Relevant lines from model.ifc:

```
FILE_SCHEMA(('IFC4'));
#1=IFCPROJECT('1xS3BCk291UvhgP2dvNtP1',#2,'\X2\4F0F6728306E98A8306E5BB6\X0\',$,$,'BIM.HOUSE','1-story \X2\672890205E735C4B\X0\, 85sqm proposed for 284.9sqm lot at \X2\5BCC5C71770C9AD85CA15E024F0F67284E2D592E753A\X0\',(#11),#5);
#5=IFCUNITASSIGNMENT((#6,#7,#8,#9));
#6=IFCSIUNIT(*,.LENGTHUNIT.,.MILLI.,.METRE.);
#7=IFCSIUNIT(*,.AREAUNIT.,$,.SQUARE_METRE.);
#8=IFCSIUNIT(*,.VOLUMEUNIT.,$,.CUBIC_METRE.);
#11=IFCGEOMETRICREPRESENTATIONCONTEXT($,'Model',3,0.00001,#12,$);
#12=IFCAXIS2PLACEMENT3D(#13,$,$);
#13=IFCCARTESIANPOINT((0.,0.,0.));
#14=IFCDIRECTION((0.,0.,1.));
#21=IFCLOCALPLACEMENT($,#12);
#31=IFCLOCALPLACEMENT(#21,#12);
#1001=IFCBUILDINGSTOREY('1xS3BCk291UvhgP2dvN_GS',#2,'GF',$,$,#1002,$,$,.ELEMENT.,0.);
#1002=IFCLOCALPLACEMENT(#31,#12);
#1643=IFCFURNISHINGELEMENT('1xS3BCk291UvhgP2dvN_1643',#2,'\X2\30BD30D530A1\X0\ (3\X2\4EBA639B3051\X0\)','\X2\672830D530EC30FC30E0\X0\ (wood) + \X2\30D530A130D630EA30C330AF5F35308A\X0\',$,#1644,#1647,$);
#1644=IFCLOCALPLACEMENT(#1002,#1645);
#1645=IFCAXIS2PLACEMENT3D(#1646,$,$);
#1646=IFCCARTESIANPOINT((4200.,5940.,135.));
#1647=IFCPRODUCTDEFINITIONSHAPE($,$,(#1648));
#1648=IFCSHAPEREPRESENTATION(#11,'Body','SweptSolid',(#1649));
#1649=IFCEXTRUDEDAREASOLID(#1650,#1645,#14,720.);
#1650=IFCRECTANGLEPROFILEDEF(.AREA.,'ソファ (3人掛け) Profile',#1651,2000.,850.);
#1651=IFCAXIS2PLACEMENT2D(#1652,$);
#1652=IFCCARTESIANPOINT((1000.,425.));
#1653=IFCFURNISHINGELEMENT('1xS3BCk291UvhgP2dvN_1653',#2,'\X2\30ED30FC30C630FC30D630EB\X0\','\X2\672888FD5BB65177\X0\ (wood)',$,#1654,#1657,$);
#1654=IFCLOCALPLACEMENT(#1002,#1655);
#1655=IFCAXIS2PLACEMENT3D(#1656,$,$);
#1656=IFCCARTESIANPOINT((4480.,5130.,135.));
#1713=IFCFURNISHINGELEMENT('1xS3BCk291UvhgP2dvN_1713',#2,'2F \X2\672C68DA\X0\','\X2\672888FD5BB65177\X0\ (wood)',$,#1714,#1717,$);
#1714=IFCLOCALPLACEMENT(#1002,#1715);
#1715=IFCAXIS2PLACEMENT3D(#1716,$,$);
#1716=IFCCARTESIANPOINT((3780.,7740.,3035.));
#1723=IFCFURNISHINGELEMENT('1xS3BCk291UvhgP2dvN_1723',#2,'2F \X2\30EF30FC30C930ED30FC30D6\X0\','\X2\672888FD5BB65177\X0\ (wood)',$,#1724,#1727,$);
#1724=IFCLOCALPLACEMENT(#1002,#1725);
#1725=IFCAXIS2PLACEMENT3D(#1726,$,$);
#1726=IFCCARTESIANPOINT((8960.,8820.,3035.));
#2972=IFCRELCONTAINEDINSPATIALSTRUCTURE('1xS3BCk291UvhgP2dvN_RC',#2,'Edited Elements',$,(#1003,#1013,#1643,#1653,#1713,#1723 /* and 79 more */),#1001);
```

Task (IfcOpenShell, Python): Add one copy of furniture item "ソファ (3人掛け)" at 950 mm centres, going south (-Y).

```python
import numpy as np
import ifcopenshell
import ifcopenshell.api.geometry
import ifcopenshell.api.root
import ifcopenshell.util.element
import ifcopenshell.util.placement
import ifcopenshell.util.unit

model = ifcopenshell.open("model.ifc")
unit_scale = ifcopenshell.util.unit.calculate_unit_scale(model)


def reuse_history(source, copy):
    """copy_class also copies each property set's owner history, people and application; keep the originals."""
    for rel in copy.IsDefinedBy:
        if rel.is_a("IfcRelDefinesByProperties") and (history := rel.RelatingPropertyDefinition.OwnerHistory):
            rel.RelatingPropertyDefinition.OwnerHistory = source.OwnerHistory
            ifcopenshell.util.element.remove_deep2(model, history)


source = model.by_guid("1xS3BCk291UvhgP2dvN_1643")
base = ifcopenshell.util.placement.get_local_placement(source.ObjectPlacement)
step = np.array([0.0, -1.0, 0.0]) * 0.95 / unit_scale

for i in range(1, 2):
    copy = ifcopenshell.api.root.copy_class(model, product=source)
    copy.Representation = ifcopenshell.util.element.copy_deep(
        model, source.Representation, exclude=["IfcGeometricRepresentationContext", "IfcRepresentationMap"]
    )
    reuse_history(source, copy)
    matrix = base.copy()
    matrix[:3, 3] += i * step
    print("added at", matrix[:3, 3].round(3) + 0.0)
    ifcopenshell.api.geometry.edit_object_placement(model, product=copy, matrix=matrix, is_si=False)

model.write("model_updated.ifc")
```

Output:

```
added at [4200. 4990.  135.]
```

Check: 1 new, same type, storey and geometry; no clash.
